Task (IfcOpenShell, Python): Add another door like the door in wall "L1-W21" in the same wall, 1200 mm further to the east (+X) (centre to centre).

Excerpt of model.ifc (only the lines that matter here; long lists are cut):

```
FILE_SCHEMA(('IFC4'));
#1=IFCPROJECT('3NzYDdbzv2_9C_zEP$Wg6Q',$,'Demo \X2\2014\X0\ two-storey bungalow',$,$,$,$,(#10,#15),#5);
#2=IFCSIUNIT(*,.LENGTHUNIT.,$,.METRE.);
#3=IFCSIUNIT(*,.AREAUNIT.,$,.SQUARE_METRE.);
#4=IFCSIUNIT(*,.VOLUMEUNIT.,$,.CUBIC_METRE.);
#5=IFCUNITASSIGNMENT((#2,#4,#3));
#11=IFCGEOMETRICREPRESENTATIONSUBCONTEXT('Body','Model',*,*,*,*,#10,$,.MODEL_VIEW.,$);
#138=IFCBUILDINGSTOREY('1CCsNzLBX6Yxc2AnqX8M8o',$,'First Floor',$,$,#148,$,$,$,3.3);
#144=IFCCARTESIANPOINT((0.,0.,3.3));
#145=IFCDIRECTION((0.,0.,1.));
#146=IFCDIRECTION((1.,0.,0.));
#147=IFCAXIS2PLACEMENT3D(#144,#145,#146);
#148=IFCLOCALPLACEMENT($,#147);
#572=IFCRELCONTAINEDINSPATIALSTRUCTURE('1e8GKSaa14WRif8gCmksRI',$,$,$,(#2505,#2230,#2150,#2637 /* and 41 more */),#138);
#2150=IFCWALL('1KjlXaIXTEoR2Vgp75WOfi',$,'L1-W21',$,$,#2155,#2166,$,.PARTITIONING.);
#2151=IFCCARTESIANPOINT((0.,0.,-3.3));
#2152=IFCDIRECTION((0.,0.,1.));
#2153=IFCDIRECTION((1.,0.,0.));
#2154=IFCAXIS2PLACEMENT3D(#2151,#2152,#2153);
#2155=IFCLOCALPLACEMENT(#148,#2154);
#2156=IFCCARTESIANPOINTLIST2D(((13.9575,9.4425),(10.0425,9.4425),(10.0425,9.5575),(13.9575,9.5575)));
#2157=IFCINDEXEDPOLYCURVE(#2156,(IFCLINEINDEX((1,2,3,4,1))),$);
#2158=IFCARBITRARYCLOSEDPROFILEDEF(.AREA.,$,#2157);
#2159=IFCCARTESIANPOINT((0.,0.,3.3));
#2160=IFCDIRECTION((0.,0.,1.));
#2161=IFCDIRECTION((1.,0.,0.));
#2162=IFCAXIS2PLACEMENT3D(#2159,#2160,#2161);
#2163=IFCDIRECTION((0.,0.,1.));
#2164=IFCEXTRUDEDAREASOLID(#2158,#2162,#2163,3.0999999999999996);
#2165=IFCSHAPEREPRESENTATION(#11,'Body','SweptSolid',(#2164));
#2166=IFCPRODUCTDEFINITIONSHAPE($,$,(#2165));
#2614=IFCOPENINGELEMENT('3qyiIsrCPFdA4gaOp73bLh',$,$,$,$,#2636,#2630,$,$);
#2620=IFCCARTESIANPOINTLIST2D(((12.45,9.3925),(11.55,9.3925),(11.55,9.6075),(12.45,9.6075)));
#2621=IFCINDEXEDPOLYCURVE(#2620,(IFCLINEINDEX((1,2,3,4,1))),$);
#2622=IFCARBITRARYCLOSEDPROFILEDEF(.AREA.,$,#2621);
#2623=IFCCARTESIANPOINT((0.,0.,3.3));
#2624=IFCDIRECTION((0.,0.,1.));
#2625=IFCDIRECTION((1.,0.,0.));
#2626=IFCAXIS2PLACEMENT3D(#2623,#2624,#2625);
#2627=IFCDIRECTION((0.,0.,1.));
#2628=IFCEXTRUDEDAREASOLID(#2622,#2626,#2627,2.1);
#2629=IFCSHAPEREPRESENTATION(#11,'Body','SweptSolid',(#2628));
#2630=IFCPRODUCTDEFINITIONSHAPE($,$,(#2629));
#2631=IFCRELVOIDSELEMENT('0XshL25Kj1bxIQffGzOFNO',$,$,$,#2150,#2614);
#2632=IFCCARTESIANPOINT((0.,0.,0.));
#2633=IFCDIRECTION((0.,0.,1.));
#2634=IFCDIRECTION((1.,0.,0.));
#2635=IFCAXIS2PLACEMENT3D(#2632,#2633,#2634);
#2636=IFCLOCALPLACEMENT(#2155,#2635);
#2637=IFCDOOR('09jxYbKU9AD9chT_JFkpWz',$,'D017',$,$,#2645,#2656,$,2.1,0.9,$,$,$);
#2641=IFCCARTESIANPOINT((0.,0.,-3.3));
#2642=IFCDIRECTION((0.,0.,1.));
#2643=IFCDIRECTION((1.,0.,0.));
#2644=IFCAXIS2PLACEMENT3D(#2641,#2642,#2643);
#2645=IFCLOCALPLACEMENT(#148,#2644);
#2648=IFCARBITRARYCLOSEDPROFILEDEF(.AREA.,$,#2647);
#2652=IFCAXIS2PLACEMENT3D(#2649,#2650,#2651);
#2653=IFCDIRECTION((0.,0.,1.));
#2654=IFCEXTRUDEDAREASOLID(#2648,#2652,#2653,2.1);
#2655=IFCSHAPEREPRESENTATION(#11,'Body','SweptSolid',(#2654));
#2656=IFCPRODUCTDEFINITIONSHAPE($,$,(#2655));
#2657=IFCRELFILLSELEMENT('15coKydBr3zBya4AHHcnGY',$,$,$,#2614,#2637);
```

```python
import ifcopenshell
import ifcopenshell.api.feature
import ifcopenshell.api.geometry
import ifcopenshell.api.root
import ifcopenshell.geom
import ifcopenshell.util.element
import ifcopenshell.util.placement
import ifcopenshell.util.shape
import ifcopenshell.util.unit

model = ifcopenshell.open("model.ifc")
unit_scale = ifcopenshell.util.unit.calculate_unit_scale(model)
settings = ifcopenshell.geom.settings()


def volume(element):
    """Net volume in cubic metres, openings subtracted."""
    shape = ifcopenshell.geom.create_shape(settings, element)
    return ifcopenshell.util.shape.get_volume(shape.geometry)


door = model.by_guid("09jxYbKU9AD9chT_JFkpWz")
opening = door.FillsVoids[0].RelatingOpeningElement
wall = opening.VoidsElements[0].RelatingBuildingElement
before = volume(wall)
shift = ifcopenshell.util.placement.get_local_placement(wall.ObjectPlacement)[:3, 0] * 1.2 / unit_scale

# copy_class copies the void relationship, type, container and properties, but no geometry.
new_opening = ifcopenshell.api.root.copy_class(model, product=opening)
new_opening.Representation = ifcopenshell.util.element.copy_deep(
    model, opening.Representation, exclude=["IfcGeometricRepresentationContext", "IfcRepresentationMap"]
)
new_door = ifcopenshell.api.root.copy_class(model, product=door)
new_door.Representation = ifcopenshell.util.element.copy_deep(
    model, door.Representation, exclude=["IfcGeometricRepresentationContext", "IfcRepresentationMap"]
)
ifcopenshell.api.feature.add_filling(model, opening=new_opening, element=new_door)

for old, new in ((opening, new_opening), (door, new_door)):
    matrix = ifcopenshell.util.placement.get_local_placement(old.ObjectPlacement)
    matrix[:3, 3] += shift
    ifcopenshell.api.geometry.edit_object_placement(model, product=new, matrix=matrix, is_si=False)

after = volume(wall)

print(f"wall volume {before:.3f} -> {after:.3f} m3")

model.write("model-out.ifc")
```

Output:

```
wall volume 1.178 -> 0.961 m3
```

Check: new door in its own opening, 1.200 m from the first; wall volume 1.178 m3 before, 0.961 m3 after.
